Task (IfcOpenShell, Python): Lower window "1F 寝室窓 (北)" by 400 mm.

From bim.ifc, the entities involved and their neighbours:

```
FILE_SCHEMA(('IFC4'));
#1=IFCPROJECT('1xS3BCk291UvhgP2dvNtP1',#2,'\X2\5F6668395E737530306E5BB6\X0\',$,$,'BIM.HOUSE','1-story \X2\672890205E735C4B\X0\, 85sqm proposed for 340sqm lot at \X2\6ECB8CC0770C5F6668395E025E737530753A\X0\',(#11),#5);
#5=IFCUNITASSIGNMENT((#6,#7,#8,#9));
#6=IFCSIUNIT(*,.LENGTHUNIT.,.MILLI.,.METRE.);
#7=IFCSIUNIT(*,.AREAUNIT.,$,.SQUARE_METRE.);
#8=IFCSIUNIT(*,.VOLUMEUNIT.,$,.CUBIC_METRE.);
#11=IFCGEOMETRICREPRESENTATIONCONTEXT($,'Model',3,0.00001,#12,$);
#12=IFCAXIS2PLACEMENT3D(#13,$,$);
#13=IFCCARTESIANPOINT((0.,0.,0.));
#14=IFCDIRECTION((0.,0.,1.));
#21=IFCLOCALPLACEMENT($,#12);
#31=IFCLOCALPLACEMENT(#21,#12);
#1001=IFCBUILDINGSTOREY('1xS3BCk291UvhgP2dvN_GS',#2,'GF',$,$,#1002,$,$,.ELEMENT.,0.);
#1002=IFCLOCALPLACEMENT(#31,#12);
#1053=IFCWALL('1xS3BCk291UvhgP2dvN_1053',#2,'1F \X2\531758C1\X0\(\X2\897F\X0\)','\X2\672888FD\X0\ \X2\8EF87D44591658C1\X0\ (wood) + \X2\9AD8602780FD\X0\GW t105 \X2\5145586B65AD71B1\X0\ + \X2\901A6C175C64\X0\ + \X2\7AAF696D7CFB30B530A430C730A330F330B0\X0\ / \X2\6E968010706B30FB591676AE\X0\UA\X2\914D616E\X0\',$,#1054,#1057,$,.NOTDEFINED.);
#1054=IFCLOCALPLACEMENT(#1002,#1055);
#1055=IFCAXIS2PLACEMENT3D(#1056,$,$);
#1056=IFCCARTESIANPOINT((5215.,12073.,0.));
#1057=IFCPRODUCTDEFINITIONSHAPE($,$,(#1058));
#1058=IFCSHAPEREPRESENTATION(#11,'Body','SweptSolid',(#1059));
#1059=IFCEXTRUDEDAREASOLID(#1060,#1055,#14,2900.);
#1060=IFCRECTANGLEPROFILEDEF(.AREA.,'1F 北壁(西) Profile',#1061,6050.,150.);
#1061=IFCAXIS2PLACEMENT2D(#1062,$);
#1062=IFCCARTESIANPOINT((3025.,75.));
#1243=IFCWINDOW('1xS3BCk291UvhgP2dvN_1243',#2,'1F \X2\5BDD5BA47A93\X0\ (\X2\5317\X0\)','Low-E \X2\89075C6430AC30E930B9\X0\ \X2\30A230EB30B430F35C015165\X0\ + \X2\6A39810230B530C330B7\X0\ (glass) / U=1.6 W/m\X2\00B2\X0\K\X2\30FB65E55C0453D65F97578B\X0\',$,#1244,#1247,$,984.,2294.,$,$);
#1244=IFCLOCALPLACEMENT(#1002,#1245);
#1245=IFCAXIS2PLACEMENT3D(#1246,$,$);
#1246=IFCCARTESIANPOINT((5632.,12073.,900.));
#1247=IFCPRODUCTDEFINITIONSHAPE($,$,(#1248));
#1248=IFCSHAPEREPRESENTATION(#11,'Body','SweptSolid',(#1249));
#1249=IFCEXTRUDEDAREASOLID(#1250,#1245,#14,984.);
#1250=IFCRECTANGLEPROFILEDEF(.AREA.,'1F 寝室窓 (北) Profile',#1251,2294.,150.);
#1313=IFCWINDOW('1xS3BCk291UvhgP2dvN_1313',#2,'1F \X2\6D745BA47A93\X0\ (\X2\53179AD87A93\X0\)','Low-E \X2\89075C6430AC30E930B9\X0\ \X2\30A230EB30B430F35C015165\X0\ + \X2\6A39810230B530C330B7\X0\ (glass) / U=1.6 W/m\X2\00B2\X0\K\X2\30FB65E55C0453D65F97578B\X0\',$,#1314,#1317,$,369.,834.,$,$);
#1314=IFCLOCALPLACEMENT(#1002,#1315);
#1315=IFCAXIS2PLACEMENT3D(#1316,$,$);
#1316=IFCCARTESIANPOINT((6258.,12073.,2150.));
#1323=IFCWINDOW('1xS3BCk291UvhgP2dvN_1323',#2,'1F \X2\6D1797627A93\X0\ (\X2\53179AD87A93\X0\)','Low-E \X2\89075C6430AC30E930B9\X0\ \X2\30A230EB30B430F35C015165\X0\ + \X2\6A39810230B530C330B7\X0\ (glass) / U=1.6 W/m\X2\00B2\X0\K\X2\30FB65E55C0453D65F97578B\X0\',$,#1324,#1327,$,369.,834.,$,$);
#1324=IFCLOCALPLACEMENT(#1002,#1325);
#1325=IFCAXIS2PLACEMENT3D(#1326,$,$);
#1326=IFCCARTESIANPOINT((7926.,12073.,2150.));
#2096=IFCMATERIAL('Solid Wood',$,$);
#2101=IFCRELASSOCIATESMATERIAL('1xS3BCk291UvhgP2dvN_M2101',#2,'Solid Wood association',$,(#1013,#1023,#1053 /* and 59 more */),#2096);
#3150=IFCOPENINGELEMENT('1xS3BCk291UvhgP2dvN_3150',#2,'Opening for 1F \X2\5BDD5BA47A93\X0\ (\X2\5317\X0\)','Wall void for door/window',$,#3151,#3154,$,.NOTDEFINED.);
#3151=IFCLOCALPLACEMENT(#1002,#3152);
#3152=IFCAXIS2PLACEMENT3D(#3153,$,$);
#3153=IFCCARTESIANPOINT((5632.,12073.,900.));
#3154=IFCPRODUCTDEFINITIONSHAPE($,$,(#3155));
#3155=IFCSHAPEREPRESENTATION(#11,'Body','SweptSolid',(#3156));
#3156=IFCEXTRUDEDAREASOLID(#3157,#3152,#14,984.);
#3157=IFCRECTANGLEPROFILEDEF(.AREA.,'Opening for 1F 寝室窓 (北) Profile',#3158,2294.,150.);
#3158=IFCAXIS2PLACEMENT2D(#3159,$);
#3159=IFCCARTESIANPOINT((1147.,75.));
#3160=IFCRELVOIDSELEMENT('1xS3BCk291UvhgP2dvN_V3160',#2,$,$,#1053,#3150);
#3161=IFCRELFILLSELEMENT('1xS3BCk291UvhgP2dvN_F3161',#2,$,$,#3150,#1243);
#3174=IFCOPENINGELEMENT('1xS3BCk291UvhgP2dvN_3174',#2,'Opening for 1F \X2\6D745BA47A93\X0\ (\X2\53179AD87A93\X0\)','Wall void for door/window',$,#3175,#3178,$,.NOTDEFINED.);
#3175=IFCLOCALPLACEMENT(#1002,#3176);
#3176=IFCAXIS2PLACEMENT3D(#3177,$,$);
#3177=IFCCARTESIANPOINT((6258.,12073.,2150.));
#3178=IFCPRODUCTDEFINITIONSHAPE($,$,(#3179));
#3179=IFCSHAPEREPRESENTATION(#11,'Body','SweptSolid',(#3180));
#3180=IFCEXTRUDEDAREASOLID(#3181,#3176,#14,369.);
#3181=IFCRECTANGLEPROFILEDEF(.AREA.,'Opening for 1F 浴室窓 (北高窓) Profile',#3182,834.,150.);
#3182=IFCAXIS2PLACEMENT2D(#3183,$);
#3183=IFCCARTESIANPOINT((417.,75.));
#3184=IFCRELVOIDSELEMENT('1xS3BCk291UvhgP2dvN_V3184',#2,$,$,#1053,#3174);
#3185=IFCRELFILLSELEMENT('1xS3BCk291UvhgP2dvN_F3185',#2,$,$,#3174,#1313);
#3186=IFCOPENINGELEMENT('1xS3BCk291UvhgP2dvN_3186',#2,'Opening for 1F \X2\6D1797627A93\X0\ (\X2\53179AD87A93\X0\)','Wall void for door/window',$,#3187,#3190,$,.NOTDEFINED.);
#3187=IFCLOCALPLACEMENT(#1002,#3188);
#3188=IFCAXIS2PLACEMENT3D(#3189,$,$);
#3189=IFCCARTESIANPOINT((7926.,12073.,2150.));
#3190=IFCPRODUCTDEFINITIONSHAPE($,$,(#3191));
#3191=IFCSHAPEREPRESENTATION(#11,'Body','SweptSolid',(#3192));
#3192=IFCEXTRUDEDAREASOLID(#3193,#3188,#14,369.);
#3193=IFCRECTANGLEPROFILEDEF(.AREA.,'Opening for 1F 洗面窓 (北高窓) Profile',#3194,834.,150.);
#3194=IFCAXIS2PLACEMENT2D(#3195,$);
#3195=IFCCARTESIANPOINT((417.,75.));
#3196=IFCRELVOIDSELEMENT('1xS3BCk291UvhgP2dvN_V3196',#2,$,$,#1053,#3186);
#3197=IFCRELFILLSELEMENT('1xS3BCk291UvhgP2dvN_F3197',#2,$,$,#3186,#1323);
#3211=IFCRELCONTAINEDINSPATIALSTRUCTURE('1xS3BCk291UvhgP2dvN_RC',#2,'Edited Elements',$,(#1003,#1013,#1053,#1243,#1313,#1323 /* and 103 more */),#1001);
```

```python
import numpy as np
import ifcopenshell
import ifcopenshell.api.geometry
import ifcopenshell.util.placement
import ifcopenshell.util.unit

model = ifcopenshell.open("bim.ifc")
unit_scale = ifcopenshell.util.unit.calculate_unit_scale(model)

window = model.by_guid("1xS3BCk291UvhgP2dvN_1243")
opening = window.FillsVoids[0].RelatingOpeningElement
dz = -0.4 / unit_scale

shift = np.array([0.0, 0.0, dz])
# The window is not placed relative to its opening, so move both.
for product in (opening, window):
    matrix = ifcopenshell.util.placement.get_local_placement(product.ObjectPlacement)
    matrix[:3, 3] += shift
    ifcopenshell.api.geometry.edit_object_placement(model, product=product, matrix=matrix, is_si=False)

print(f"moved by {dz * unit_scale:+.3f} m")

model.write("bim_updated.ifc")
```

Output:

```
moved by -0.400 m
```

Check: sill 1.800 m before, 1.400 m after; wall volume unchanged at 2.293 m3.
